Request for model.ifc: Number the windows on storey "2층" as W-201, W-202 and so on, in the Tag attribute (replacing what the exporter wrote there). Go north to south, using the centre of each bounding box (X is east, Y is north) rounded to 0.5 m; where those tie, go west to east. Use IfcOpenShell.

First a look at what the model holds.

```python
import ifcopenshell
import ifcopenshell.util.element
import ifcopenshell.util.placement

model = ifcopenshell.open("model.ifc")
print(model.schema)
storey = next(s for s in model.by_type("IfcBuildingStorey") if s.Name == "2층")
windows = [e for e in ifcopenshell.util.element.get_decomposition(storey) if e.is_a("IfcWindow")]
for e in sorted(windows, key=lambda e: e.id()):
    origin = ifcopenshell.util.placement.get_local_placement(e.ObjectPlacement)[:3, 3]
    print(e.id(), e.Tag, e.Name, origin.round(2) + 0.0, sep=" | ")
```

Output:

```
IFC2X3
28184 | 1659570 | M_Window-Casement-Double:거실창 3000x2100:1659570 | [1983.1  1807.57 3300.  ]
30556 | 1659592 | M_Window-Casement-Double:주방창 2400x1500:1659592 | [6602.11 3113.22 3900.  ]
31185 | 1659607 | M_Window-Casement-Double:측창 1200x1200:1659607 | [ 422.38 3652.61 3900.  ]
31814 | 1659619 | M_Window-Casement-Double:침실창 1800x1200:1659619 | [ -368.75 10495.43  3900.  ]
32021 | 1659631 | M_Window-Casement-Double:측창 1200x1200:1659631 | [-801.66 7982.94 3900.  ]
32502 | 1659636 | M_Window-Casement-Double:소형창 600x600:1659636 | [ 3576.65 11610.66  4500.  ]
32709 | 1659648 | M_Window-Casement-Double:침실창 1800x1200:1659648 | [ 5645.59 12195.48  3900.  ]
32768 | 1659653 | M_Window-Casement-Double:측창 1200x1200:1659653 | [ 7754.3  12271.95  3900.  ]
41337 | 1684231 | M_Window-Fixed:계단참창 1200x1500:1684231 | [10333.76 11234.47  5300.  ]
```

```python
import ifcopenshell
import ifcopenshell.geom
import ifcopenshell.util.element
import ifcopenshell.util.shape

model = ifcopenshell.open("model.ifc")
settings = ifcopenshell.geom.settings()
settings.set("use-world-coords", True)


def centre(element):
    shape = ifcopenshell.geom.create_shape(settings, element)
    return ifcopenshell.util.shape.get_bbox_centroid(shape.geometry)


storey = next(s for s in model.by_type("IfcBuildingStorey") if s.Name == "2층")
windows = [e for e in ifcopenshell.util.element.get_decomposition(storey) if e.is_a("IfcWindow")]

# Insertion points can sit at a corner or the storey origin, so sort by the geometry (in metres).
centres = {e: centre(e) for e in windows}
windows.sort(key=lambda e: (-round(centres[e][1] / 0.5), centres[e][0]))

for i, e in enumerate(windows, start=1):
    number = f"W-2{i:02d}"
    e.Tag = number
    print(e.id(), number)

model.write("model_rev.ifc")
```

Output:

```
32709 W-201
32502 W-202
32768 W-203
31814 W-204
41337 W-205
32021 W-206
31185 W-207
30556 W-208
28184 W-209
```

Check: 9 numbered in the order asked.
